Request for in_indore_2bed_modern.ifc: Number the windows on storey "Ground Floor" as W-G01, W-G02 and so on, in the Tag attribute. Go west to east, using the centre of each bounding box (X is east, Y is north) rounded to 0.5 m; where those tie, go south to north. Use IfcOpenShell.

First a look at what the model holds.

```python
import ifcopenshell
import ifcopenshell.util.element
import ifcopenshell.util.placement

model = ifcopenshell.open("in_indore_2bed_modern.ifc")
print(model.schema)
storey = next(s for s in model.by_type("IfcBuildingStorey") if s.Name == "Ground Floor")
windows = [e for e in ifcopenshell.util.element.get_decomposition(storey) if e.is_a("IfcWindow")]
for e in sorted(windows, key=lambda e: e.id()):
    origin = ifcopenshell.util.placement.get_local_placement(e.ObjectPlacement)[:3, 3]
    print(e.id(), e.Tag, e.Name, origin.round(2) + 0.0, sep=" | ")
```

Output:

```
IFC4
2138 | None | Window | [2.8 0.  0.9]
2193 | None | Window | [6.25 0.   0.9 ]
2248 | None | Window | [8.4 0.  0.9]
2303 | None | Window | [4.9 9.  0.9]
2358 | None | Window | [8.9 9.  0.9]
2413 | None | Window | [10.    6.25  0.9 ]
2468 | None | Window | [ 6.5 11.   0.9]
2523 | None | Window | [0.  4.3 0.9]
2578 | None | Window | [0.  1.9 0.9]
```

```python
import ifcopenshell
import ifcopenshell.geom
import ifcopenshell.util.element
import ifcopenshell.util.shape

model = ifcopenshell.open("in_indore_2bed_modern.ifc")
settings = ifcopenshell.geom.settings()
settings.set("use-world-coords", True)


def centre(element):
    shape = ifcopenshell.geom.create_shape(settings, element)
    return ifcopenshell.util.shape.get_bbox_centroid(shape.geometry)


storey = next(s for s in model.by_type("IfcBuildingStorey") if s.Name == "Ground Floor")
windows = [e for e in ifcopenshell.util.element.get_decomposition(storey) if e.is_a("IfcWindow")]

# Insertion points can sit at a corner or the storey origin, so sort by the geometry (in metres).
centres = {e: centre(e) for e in windows}
windows.sort(key=lambda e: (round(centres[e][0] / 0.5), centres[e][1]))

for i, e in enumerate(windows, start=1):
    number = f"W-G{i:02d}"
    e.Tag = number
    print(e.id(), number)

model.write("in_indore_2bed_modern-out.ifc")
```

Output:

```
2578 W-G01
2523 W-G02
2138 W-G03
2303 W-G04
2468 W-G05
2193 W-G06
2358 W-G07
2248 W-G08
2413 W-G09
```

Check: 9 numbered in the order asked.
